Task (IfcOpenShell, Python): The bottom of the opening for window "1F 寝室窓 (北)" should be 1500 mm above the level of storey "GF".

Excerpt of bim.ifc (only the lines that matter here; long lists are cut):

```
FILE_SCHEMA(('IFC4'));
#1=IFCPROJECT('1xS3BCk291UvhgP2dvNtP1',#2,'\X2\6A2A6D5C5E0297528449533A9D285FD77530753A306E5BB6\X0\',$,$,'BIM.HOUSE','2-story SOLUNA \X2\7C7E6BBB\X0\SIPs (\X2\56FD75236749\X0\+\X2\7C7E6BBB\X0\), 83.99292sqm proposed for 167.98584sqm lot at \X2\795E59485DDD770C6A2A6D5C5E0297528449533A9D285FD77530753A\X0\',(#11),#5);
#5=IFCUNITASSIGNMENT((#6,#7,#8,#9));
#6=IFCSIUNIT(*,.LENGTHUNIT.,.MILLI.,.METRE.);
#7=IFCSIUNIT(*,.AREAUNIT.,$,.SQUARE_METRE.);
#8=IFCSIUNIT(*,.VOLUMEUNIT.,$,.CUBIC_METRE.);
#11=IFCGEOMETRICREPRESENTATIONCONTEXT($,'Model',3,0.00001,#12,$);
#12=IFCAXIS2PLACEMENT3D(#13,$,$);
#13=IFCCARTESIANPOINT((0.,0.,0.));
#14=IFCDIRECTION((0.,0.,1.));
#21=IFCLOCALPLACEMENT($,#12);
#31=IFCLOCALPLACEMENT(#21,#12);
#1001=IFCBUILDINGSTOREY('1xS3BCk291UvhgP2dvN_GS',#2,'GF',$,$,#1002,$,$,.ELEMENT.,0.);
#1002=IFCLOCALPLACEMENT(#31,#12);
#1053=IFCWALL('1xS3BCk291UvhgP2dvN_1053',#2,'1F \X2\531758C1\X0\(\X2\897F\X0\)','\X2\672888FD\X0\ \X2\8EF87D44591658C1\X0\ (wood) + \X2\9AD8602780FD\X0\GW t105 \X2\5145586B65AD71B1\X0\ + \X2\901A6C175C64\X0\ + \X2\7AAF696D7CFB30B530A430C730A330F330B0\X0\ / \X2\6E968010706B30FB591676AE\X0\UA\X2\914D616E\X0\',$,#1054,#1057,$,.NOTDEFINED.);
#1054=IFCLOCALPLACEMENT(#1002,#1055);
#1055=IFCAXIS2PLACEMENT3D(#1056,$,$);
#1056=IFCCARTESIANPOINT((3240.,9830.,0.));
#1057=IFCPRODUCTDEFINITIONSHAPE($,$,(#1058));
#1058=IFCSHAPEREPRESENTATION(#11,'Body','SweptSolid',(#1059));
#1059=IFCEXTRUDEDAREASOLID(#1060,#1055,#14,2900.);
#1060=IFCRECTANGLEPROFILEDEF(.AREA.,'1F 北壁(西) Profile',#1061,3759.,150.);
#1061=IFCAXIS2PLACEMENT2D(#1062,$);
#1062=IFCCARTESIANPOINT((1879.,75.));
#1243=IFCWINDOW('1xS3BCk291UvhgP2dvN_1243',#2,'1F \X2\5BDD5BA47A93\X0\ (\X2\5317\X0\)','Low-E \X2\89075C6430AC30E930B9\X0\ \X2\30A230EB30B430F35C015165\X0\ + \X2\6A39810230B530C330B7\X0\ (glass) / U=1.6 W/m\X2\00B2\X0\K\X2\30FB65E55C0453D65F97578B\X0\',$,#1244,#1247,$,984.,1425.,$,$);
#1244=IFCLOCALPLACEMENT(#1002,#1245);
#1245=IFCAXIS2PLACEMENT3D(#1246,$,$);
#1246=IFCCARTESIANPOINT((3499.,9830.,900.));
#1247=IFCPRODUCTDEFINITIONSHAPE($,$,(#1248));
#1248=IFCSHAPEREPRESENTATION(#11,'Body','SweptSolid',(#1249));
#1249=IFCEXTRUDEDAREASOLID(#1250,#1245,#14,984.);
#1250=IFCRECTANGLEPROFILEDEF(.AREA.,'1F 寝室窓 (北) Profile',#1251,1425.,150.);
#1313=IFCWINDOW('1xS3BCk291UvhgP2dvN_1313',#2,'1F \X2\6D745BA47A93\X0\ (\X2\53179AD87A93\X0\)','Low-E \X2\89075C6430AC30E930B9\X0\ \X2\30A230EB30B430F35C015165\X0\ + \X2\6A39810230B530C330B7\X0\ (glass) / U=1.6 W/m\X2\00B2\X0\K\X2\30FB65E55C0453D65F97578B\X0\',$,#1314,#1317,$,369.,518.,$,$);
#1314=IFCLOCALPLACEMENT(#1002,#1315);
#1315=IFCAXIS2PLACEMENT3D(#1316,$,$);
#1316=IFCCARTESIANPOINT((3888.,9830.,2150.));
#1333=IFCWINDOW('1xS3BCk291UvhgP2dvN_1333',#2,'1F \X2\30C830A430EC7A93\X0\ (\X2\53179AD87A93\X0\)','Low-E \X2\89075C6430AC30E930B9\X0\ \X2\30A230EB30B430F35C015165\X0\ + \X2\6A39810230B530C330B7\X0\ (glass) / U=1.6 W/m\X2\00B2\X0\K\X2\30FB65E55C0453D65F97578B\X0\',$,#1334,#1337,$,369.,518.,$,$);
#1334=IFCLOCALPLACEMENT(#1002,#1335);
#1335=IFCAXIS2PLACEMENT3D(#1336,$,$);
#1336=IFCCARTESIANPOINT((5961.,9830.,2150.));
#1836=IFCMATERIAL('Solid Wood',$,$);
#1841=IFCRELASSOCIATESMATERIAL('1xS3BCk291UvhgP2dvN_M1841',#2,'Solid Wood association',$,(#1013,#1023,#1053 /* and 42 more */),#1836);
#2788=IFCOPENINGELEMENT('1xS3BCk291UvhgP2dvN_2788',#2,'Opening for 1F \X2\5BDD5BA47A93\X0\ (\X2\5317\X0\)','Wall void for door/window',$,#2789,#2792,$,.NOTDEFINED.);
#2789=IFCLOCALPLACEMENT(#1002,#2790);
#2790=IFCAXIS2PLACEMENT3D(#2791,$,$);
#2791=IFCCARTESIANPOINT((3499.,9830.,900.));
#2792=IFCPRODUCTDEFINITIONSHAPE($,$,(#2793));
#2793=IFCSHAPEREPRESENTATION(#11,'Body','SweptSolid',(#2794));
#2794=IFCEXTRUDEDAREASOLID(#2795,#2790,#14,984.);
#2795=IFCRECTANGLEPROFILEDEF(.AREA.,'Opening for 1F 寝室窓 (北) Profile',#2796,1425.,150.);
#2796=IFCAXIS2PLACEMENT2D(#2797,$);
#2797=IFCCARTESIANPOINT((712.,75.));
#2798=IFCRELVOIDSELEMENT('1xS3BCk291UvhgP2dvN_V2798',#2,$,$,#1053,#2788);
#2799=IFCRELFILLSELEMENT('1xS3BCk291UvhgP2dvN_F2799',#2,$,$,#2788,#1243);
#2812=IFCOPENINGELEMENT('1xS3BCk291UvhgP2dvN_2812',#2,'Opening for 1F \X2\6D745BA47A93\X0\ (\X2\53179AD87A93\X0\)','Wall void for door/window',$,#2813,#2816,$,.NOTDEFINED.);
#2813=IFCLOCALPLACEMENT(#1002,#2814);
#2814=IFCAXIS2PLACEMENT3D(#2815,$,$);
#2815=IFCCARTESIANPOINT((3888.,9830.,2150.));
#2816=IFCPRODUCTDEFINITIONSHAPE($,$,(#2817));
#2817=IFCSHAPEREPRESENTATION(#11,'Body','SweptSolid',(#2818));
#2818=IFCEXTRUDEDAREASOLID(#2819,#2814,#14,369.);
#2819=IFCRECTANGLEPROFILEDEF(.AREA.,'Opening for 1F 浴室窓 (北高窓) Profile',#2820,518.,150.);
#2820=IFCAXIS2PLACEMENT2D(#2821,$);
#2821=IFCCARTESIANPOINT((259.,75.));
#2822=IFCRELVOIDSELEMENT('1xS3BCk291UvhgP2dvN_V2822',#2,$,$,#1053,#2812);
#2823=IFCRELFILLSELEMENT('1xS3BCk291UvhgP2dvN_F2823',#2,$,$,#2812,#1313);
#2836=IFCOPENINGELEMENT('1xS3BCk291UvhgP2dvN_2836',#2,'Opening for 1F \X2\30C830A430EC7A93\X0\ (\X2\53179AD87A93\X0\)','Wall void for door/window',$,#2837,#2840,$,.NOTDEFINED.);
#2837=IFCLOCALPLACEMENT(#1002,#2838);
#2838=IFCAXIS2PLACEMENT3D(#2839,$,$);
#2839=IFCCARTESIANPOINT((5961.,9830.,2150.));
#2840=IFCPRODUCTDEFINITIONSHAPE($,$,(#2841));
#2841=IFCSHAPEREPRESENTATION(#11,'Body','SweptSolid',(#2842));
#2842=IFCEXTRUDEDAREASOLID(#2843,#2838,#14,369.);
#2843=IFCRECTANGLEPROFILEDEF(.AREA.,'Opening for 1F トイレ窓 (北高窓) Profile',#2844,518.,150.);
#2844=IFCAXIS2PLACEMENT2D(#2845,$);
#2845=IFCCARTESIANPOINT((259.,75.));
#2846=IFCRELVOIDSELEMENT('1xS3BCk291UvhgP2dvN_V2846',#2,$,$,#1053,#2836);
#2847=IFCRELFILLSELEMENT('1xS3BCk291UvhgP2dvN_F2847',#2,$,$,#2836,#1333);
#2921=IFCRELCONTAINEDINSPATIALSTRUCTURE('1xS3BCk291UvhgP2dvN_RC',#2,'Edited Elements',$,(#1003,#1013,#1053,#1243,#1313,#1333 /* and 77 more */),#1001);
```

```python
import numpy as np
import ifcopenshell
import ifcopenshell.api.geometry
import ifcopenshell.geom
import ifcopenshell.util.element
import ifcopenshell.util.placement
import ifcopenshell.util.shape
import ifcopenshell.util.unit

model = ifcopenshell.open("bim.ifc")
unit_scale = ifcopenshell.util.unit.calculate_unit_scale(model)

window = model.by_id(1243)
opening = window.FillsVoids[0].RelatingOpeningElement
storey = ifcopenshell.util.element.get_container(window, ifc_class="IfcBuildingStorey")
level = ifcopenshell.util.placement.get_local_placement(storey.ObjectPlacement)[2, 3]

# The opening's origin need not be at the sill, so measure its lowest point.
shape = ifcopenshell.geom.create_shape(ifcopenshell.geom.settings(), opening)
bottom = ifcopenshell.util.shape.get_shape_bottom_elevation(shape, shape.geometry) / unit_scale
dz = level + 1.5 / unit_scale - bottom

shift = np.array([0.0, 0.0, dz])
# The window is not placed relative to its opening, so move both.
for product in (opening, window):
    matrix = ifcopenshell.util.placement.get_local_placement(product.ObjectPlacement)
    matrix[:3, 3] += shift
    ifcopenshell.api.geometry.edit_object_placement(model, product=product, matrix=matrix, is_si=False)

print(f"moved by {dz * unit_scale:+.3f} m")

model.write("bim_updated.ifc")
```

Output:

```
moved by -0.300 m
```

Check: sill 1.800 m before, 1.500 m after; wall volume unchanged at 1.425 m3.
